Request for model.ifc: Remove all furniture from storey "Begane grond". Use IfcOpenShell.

First a look at what the model holds.

```python
import ifcopenshell
import ifcopenshell.util.element

model = ifcopenshell.open("model.ifc")
print(model.schema)
storey = next(s for s in model.by_type("IfcBuildingStorey") if s.Name == "Begane grond")
furniture = [e for e in ifcopenshell.util.element.get_decomposition(storey) if e.is_a("IfcFurnishingElement")]
seen = {}
for e in furniture:
    element_type = ifcopenshell.util.element.get_type(e)
    name = element_type.Name if element_type not in (None, e) else None
    seen[name] = seen.get(name, 0) + 1
for name, count in sorted(seen.items(), key=str):
    print(count, "x", name)
```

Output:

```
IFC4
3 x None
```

```python
import ifcopenshell
import ifcopenshell.api.root
import ifcopenshell.util.element

model = ifcopenshell.open("model.ifc")

storey = next(s for s in model.by_type("IfcBuildingStorey") if s.Name == "Begane grond")
furniture = [e for e in ifcopenshell.util.element.get_decomposition(storey) if e.is_a("IfcFurnishingElement")]

for e in furniture:
    ifcopenshell.api.root.remove_product(model, product=e)
print(len(furniture), "removed")

model.write("model-out.ifc")
```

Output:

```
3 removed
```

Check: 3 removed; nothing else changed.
